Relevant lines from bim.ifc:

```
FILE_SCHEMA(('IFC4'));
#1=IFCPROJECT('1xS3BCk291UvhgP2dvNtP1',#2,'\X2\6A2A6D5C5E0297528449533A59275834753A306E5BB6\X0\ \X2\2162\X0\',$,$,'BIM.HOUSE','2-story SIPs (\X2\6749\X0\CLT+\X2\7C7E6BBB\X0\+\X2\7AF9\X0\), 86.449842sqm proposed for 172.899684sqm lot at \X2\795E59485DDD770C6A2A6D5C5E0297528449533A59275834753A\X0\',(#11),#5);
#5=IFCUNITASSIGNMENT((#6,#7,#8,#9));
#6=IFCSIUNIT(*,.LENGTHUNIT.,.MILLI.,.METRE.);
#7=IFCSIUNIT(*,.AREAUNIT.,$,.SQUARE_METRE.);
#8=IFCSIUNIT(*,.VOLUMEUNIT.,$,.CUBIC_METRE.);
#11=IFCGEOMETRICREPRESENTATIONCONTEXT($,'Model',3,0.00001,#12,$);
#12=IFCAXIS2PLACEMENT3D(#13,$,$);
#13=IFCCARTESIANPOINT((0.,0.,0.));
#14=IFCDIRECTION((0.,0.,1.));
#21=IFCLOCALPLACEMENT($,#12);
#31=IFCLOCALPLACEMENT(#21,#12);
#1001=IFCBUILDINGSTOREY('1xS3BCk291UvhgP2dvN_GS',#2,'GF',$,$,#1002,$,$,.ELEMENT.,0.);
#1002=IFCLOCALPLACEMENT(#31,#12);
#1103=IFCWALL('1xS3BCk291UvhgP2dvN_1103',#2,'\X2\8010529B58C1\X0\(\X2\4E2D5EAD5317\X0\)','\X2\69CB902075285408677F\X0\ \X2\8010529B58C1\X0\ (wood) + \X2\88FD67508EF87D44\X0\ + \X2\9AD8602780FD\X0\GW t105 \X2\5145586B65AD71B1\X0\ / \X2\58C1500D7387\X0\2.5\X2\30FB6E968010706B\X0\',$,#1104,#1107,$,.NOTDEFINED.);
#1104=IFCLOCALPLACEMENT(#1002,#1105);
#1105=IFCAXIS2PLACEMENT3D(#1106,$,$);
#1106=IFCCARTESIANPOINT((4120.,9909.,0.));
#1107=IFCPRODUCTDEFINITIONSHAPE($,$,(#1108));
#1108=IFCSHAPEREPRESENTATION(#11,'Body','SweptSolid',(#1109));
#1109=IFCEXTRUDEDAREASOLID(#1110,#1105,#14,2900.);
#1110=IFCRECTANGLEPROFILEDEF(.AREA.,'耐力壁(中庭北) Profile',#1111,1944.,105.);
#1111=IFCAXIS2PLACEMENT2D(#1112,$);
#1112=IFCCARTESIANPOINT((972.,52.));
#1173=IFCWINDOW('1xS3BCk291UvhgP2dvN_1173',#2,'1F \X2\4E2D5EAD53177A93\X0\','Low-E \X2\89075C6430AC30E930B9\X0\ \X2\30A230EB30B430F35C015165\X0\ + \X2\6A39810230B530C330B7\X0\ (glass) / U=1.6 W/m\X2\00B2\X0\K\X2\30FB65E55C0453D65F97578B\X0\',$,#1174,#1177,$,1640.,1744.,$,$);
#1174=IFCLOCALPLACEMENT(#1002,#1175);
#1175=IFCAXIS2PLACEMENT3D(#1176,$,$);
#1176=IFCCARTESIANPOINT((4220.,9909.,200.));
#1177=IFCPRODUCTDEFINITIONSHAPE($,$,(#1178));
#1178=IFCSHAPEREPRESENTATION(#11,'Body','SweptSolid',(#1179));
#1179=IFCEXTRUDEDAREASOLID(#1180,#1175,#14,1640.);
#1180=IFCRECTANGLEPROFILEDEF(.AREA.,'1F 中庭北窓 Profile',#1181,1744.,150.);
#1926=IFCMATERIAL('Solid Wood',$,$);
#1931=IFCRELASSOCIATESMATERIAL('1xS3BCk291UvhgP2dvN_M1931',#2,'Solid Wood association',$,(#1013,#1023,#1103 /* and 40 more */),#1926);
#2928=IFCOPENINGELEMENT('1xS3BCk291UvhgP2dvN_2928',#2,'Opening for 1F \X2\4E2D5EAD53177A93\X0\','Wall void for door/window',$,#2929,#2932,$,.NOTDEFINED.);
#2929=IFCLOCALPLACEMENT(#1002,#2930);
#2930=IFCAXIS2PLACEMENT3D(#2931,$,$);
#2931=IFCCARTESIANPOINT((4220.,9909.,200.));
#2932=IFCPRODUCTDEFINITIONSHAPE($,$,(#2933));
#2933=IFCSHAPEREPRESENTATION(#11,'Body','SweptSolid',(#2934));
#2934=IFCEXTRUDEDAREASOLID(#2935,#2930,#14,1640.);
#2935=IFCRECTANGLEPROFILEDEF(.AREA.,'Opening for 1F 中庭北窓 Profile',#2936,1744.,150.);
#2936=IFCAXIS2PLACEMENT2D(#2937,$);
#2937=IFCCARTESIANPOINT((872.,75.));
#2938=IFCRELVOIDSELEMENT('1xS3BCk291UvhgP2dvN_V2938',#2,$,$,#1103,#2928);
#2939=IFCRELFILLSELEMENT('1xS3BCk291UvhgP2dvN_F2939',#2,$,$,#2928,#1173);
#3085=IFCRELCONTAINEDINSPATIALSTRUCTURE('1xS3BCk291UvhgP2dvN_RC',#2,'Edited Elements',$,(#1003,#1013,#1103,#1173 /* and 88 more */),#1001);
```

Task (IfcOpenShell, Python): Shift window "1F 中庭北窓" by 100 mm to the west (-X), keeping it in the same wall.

```python
import ifcopenshell
import ifcopenshell.api.geometry
import ifcopenshell.util.placement
import ifcopenshell.util.unit

model = ifcopenshell.open("bim.ifc")
unit_scale = ifcopenshell.util.unit.calculate_unit_scale(model)

window = model.by_guid("1xS3BCk291UvhgP2dvN_1173")
opening = window.FillsVoids[0].RelatingOpeningElement
wall = opening.VoidsElements[0].RelatingBuildingElement

wall_matrix = ifcopenshell.util.placement.get_local_placement(wall.ObjectPlacement)
shift = wall_matrix[:3, 0] * -0.1 / unit_scale
before = ifcopenshell.util.placement.get_local_placement(window.ObjectPlacement)[:3, 3].copy()

# The window is not placed relative to its opening, so move both.
for product in (opening, window):
    matrix = ifcopenshell.util.placement.get_local_placement(product.ObjectPlacement)
    matrix[:3, 3] += shift
    ifcopenshell.api.geometry.edit_object_placement(model, product=product, matrix=matrix, is_si=False)

after = ifcopenshell.util.placement.get_local_placement(window.ObjectPlacement)[:3, 3]
print("window moved by", (after - before).round(3) + 0.0)

model.write("bim_rev.ifc")
```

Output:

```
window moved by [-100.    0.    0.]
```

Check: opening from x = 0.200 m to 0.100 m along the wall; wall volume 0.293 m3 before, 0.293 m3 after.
